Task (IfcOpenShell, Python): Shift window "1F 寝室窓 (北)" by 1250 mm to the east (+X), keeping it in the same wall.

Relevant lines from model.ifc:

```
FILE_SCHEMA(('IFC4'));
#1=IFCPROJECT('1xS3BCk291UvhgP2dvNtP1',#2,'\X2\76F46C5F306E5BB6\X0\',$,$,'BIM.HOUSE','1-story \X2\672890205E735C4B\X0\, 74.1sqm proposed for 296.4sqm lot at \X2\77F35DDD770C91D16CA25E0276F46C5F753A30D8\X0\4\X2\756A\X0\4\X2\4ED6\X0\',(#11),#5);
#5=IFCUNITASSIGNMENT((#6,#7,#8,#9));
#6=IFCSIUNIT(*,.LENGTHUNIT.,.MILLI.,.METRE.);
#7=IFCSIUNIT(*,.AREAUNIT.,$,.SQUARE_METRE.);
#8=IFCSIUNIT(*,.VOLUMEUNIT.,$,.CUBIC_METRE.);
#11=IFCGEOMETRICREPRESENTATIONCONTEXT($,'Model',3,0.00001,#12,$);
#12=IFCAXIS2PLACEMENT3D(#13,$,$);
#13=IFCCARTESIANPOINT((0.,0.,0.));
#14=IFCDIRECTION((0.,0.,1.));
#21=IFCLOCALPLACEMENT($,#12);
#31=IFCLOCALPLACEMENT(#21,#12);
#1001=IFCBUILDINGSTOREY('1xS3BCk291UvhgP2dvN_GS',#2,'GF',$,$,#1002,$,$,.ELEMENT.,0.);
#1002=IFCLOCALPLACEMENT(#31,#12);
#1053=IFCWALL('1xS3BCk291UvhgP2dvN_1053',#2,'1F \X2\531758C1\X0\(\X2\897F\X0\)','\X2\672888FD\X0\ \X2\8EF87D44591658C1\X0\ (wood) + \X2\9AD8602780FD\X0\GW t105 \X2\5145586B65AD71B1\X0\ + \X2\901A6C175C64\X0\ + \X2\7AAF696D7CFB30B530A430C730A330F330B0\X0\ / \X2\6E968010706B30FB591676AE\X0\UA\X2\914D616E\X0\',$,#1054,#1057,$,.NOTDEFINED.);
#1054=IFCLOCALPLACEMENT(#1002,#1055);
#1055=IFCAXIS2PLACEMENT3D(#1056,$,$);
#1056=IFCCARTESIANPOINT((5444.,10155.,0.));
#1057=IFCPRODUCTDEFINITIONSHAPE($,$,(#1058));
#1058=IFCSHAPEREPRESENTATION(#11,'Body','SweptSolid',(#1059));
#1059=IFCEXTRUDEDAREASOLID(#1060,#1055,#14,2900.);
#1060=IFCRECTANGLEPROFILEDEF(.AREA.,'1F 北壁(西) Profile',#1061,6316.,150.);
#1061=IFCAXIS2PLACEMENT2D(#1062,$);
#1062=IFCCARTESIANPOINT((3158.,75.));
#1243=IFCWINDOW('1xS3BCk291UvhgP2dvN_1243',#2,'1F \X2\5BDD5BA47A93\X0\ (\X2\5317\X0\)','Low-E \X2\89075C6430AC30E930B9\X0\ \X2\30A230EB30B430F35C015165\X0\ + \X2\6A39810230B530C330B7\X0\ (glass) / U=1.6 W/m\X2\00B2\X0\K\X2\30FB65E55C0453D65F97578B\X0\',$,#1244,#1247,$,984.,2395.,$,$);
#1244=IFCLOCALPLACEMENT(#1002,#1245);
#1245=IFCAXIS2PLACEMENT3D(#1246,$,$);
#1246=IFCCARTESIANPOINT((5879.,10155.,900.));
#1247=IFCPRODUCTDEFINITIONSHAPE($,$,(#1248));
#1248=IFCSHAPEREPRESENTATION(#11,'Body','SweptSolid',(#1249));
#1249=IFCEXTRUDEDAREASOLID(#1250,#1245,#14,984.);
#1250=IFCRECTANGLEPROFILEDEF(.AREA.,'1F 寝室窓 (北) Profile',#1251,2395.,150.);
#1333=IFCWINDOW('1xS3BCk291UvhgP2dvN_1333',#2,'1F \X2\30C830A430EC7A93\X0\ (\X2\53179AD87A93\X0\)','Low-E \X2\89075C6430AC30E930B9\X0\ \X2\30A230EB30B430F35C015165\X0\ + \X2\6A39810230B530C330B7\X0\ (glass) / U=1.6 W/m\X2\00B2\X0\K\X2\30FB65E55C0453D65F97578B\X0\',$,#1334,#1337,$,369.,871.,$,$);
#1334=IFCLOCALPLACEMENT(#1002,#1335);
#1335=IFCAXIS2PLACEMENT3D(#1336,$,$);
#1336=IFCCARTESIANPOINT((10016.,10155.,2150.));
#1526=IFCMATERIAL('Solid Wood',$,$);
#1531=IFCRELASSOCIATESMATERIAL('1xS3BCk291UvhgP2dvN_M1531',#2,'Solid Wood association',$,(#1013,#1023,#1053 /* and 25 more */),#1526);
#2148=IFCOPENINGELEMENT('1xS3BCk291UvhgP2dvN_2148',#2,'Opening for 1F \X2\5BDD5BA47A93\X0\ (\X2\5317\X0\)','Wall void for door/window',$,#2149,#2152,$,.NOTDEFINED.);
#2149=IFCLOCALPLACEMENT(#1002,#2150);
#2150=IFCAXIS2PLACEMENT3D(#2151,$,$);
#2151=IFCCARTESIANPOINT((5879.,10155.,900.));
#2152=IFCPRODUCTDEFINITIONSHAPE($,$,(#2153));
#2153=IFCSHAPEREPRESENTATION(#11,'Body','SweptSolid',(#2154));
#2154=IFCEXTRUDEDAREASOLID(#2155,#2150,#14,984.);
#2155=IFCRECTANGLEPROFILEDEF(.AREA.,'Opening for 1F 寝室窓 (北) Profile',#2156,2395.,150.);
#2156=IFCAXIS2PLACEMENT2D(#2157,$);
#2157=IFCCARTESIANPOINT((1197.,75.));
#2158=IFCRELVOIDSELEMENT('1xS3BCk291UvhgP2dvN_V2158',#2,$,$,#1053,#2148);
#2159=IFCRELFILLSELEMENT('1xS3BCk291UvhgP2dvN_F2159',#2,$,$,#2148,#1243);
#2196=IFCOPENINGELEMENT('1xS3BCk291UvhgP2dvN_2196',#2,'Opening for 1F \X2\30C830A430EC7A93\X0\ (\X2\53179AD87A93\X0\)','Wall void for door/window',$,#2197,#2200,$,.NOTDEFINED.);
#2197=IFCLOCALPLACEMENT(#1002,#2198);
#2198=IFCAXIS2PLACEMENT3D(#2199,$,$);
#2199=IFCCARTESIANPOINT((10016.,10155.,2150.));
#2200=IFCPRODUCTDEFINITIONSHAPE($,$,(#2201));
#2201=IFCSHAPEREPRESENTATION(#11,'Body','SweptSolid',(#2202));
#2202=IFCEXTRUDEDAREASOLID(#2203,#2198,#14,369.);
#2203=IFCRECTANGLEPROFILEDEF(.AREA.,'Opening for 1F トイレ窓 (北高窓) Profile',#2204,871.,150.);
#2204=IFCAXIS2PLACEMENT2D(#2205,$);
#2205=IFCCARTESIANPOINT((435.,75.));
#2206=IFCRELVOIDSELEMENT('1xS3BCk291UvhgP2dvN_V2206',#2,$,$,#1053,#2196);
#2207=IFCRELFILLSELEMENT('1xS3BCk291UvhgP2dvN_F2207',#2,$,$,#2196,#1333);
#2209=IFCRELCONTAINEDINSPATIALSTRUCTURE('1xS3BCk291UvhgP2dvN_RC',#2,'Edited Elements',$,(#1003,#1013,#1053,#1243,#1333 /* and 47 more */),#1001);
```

```python
import ifcopenshell
import ifcopenshell.api.geometry
import ifcopenshell.util.placement

model = ifcopenshell.open("model.ifc")

window = model.by_guid("1xS3BCk291UvhgP2dvN_1243")
opening = window.FillsVoids[0].RelatingOpeningElement
wall = opening.VoidsElements[0].RelatingBuildingElement

wall_matrix = ifcopenshell.util.placement.get_local_placement(wall.ObjectPlacement)
shift = wall_matrix[:3, 0] * 1250.0
before = ifcopenshell.util.placement.get_local_placement(window.ObjectPlacement)[:3, 3].copy()

# The window is not placed relative to its opening, so move both.
for product in (opening, window):
    matrix = ifcopenshell.util.placement.get_local_placement(product.ObjectPlacement)
    matrix[:3, 3] += shift
    ifcopenshell.api.geometry.edit_object_placement(model, product=product, matrix=matrix, is_si=False)

after = ifcopenshell.util.placement.get_local_placement(window.ObjectPlacement)[:3, 3]
print("window moved by", (after - before).round(3) + 0.0)

model.write("model_rev.ifc")
```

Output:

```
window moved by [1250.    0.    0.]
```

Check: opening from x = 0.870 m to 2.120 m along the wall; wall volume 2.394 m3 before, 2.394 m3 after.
